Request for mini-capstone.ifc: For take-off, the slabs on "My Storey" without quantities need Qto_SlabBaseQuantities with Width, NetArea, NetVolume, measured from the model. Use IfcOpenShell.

First a look at what the model holds.

```python
import ifcopenshell
import ifcopenshell.util.element
import ifcopenshell.util.unit

model = ifcopenshell.open("mini-capstone.ifc")
print(model.schema)
for unit_type in ("LENGTHUNIT", "AREAUNIT", "VOLUMEUNIT"):
    print(unit_type, ifcopenshell.util.unit.calculate_unit_scale(model, unit_type))
storey = next(s for s in model.by_type("IfcBuildingStorey") if s.Name == "My Storey")
slabs = [e for e in ifcopenshell.util.element.get_decomposition(storey) if e.is_a("IfcSlab")]
for e in sorted(slabs, key=lambda e: e.id()):
    print(e.id(), e.is_a(), e.Name, list(ifcopenshell.util.element.get_psets(e, qtos_only=True)), sep=" | ")
```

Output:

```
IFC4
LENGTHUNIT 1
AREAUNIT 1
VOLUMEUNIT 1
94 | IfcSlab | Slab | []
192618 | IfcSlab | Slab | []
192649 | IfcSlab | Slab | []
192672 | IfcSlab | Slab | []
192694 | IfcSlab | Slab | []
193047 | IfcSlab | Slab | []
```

```python
import ifcopenshell
import ifcopenshell.api.pset
import ifcopenshell.geom
import ifcopenshell.util.element
import ifcopenshell.util.shape
import ifcopenshell.util.unit

model = ifcopenshell.open("mini-capstone.ifc")
unit_scale = ifcopenshell.util.unit.calculate_unit_scale(model)
area_scale = ifcopenshell.util.unit.calculate_unit_scale(model, "AREAUNIT")
volume_scale = ifcopenshell.util.unit.calculate_unit_scale(model, "VOLUMEUNIT")
settings = ifcopenshell.geom.settings()

storey = next(s for s in model.by_type("IfcBuildingStorey") if s.Name == "My Storey")
slabs = [e for e in ifcopenshell.util.element.get_decomposition(storey) if e.is_a("IfcSlab")]

for e in sorted(slabs, key=lambda e: e.id()):
    if ifcopenshell.util.element.get_psets(e, qtos_only=True, should_inherit=False):
        continue
    # Geometry comes back in metres, in the element's own axes.
    shape = ifcopenshell.geom.create_shape(settings, e)
    values = {
        "Width": ifcopenshell.util.shape.get_z(shape.geometry) / unit_scale,
        "NetArea": ifcopenshell.util.shape.get_footprint_area(shape.geometry) / area_scale,
        "NetVolume": ifcopenshell.util.shape.get_volume(shape.geometry) / volume_scale,
    }
    qto = ifcopenshell.api.pset.add_qto(model, product=e, name="Qto_SlabBaseQuantities")
    ifcopenshell.api.pset.edit_qto(model, qto=qto, properties=values)
    print(e.id(), {k: round(v, 3) for k, v in values.items()})

model.write("mini-capstone-out.ifc")
```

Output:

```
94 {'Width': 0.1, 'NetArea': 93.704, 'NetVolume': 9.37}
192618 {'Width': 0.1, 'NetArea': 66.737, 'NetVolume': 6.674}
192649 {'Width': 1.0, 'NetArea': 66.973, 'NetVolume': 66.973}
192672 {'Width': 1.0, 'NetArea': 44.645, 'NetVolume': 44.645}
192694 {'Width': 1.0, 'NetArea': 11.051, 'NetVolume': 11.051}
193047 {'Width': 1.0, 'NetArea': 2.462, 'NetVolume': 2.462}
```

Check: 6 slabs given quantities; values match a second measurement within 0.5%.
